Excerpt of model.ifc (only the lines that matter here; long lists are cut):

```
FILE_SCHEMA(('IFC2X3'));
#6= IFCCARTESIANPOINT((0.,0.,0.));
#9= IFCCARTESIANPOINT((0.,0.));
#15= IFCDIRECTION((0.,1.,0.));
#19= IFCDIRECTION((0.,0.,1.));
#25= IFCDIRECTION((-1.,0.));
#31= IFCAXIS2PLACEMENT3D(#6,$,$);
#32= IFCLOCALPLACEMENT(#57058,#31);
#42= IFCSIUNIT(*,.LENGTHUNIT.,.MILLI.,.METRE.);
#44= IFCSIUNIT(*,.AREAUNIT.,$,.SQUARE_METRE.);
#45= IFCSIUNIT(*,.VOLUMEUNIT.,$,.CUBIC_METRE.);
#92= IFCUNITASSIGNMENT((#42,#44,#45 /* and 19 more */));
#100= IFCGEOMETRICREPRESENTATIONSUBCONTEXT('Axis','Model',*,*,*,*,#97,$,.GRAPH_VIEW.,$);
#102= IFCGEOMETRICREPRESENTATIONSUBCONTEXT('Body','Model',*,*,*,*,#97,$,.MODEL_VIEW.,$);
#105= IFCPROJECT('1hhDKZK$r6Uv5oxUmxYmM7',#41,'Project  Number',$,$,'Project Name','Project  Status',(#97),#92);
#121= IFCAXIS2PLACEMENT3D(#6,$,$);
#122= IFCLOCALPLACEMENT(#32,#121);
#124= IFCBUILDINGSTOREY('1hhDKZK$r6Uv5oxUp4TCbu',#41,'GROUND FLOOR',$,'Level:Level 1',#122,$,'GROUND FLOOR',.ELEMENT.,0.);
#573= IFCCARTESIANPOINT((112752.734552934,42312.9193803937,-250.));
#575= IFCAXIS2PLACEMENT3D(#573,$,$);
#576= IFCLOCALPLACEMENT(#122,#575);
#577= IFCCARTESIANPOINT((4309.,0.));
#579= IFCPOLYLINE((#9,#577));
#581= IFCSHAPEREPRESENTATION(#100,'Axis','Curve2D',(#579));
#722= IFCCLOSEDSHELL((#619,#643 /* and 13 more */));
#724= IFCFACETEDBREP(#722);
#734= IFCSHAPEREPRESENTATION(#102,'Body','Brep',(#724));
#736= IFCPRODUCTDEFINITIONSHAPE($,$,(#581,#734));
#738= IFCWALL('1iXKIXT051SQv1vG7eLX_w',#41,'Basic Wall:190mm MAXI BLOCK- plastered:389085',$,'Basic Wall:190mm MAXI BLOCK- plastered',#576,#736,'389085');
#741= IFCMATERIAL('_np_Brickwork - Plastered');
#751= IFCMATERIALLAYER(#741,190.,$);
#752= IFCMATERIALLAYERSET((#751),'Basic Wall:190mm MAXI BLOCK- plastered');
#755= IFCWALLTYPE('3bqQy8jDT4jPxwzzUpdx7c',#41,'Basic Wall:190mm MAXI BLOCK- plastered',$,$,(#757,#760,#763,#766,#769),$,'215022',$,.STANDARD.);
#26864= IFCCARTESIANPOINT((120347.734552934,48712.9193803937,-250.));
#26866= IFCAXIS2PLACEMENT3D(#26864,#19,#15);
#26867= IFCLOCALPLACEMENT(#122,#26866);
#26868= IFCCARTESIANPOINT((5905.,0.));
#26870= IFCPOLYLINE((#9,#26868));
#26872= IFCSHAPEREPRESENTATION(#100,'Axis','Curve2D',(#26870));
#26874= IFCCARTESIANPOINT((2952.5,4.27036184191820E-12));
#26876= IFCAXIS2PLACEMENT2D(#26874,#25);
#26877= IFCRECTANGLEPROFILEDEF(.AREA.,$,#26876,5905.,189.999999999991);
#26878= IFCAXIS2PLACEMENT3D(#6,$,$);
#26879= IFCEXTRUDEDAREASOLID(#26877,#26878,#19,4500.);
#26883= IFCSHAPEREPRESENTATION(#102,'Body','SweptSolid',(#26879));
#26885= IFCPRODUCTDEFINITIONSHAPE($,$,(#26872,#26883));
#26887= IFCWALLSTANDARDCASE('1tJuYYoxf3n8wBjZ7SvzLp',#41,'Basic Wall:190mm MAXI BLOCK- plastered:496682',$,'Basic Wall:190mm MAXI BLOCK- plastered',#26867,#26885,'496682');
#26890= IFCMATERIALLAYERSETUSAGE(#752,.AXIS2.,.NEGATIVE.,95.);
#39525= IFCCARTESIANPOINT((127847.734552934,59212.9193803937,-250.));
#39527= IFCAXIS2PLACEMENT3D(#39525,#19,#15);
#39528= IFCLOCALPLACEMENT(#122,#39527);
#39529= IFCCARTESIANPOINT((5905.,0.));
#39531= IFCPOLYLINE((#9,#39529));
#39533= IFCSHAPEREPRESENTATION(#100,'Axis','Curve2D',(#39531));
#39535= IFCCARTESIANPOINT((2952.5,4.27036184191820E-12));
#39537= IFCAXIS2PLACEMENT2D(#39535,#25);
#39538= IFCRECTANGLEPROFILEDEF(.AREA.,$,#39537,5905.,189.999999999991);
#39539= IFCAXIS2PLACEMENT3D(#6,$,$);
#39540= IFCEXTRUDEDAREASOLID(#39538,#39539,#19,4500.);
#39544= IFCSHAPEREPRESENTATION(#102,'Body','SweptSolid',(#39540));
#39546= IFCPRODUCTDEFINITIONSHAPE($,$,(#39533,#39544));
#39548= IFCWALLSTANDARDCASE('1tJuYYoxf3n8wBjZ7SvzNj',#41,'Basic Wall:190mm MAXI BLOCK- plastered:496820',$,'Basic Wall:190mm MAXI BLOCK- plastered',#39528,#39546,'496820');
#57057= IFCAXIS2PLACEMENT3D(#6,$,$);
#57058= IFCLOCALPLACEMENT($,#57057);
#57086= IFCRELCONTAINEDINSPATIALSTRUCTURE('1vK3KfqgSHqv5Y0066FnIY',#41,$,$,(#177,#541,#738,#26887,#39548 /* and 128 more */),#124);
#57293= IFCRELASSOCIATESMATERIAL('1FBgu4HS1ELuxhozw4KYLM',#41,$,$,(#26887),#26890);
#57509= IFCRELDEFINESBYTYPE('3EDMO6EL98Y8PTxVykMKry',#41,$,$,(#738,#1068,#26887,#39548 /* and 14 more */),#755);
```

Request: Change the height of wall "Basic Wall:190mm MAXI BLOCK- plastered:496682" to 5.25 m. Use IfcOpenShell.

```python
import ifcopenshell
import ifcopenshell.geom
import ifcopenshell.util.representation
import ifcopenshell.util.shape

model = ifcopenshell.open("model.ifc")
settings = ifcopenshell.geom.settings()


def volume(element):
    """Net volume in cubic metres, openings subtracted."""
    shape = ifcopenshell.geom.create_shape(settings, element)
    return ifcopenshell.util.shape.get_volume(shape.geometry)


wall = model.by_guid("1tJuYYoxf3n8wBjZ7SvzLp")
before = volume(wall)

body = ifcopenshell.util.representation.get_representation(wall, "Model", "Body")
solid = body.Items[0]
old_height = solid.Depth
solid.Depth = 5250.0
after = volume(wall)

print(f"height {old_height:g} -> {solid.Depth:g}, volume {before:.3f} -> {after:.3f} m3")

model.write("model_v2.ifc")
```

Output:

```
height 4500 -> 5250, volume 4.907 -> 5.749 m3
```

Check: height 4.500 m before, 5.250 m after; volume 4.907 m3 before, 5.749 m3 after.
